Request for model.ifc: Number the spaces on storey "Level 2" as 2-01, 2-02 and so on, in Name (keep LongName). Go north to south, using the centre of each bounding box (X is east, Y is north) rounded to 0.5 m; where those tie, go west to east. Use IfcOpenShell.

First a look at what the model holds.

```python
import ifcopenshell
import ifcopenshell.util.element
import ifcopenshell.util.placement

model = ifcopenshell.open("model.ifc")
print(model.schema)
storey = next(s for s in model.by_type("IfcBuildingStorey") if s.Name == "Level 2")
spaces = [e for e in ifcopenshell.util.element.get_decomposition(storey) if e.is_a("IfcSpace")]
for e in sorted(spaces, key=lambda e: e.id()):
    origin = ifcopenshell.util.placement.get_local_placement(e.ObjectPlacement)[:3, 3]
    print(e.id(), e.Name, e.LongName, origin.round(2) + 0.0, sep=" | ")
```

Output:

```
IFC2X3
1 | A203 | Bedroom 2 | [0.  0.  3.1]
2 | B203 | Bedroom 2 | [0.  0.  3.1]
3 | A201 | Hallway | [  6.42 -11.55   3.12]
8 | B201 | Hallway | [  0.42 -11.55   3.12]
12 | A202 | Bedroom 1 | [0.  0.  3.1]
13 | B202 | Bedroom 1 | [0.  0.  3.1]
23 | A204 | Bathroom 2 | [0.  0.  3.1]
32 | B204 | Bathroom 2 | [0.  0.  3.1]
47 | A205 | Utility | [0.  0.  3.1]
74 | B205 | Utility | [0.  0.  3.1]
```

```python
import ifcopenshell
import ifcopenshell.geom
import ifcopenshell.util.element
import ifcopenshell.util.shape

model = ifcopenshell.open("model.ifc")
settings = ifcopenshell.geom.settings()
settings.set("use-world-coords", True)


def centre(element):
    shape = ifcopenshell.geom.create_shape(settings, element)
    return ifcopenshell.util.shape.get_bbox_centroid(shape.geometry)


storey = next(s for s in model.by_type("IfcBuildingStorey") if s.Name == "Level 2")
spaces = [e for e in ifcopenshell.util.element.get_decomposition(storey) if e.is_a("IfcSpace")]

# Insertion points can sit at a corner or the storey origin, so sort by the geometry (in metres).
centres = {e: centre(e) for e in spaces}
spaces.sort(key=lambda e: (-round(centres[e][1] / 0.5), centres[e][0]))

for i, e in enumerate(spaces, start=1):
    number = f"2-{i:02d}"
    e.Name = number
    print(e.id(), number)

model.write("model_edited.ifc")
```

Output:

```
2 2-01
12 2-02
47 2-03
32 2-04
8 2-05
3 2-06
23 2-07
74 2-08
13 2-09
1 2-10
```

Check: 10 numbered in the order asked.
